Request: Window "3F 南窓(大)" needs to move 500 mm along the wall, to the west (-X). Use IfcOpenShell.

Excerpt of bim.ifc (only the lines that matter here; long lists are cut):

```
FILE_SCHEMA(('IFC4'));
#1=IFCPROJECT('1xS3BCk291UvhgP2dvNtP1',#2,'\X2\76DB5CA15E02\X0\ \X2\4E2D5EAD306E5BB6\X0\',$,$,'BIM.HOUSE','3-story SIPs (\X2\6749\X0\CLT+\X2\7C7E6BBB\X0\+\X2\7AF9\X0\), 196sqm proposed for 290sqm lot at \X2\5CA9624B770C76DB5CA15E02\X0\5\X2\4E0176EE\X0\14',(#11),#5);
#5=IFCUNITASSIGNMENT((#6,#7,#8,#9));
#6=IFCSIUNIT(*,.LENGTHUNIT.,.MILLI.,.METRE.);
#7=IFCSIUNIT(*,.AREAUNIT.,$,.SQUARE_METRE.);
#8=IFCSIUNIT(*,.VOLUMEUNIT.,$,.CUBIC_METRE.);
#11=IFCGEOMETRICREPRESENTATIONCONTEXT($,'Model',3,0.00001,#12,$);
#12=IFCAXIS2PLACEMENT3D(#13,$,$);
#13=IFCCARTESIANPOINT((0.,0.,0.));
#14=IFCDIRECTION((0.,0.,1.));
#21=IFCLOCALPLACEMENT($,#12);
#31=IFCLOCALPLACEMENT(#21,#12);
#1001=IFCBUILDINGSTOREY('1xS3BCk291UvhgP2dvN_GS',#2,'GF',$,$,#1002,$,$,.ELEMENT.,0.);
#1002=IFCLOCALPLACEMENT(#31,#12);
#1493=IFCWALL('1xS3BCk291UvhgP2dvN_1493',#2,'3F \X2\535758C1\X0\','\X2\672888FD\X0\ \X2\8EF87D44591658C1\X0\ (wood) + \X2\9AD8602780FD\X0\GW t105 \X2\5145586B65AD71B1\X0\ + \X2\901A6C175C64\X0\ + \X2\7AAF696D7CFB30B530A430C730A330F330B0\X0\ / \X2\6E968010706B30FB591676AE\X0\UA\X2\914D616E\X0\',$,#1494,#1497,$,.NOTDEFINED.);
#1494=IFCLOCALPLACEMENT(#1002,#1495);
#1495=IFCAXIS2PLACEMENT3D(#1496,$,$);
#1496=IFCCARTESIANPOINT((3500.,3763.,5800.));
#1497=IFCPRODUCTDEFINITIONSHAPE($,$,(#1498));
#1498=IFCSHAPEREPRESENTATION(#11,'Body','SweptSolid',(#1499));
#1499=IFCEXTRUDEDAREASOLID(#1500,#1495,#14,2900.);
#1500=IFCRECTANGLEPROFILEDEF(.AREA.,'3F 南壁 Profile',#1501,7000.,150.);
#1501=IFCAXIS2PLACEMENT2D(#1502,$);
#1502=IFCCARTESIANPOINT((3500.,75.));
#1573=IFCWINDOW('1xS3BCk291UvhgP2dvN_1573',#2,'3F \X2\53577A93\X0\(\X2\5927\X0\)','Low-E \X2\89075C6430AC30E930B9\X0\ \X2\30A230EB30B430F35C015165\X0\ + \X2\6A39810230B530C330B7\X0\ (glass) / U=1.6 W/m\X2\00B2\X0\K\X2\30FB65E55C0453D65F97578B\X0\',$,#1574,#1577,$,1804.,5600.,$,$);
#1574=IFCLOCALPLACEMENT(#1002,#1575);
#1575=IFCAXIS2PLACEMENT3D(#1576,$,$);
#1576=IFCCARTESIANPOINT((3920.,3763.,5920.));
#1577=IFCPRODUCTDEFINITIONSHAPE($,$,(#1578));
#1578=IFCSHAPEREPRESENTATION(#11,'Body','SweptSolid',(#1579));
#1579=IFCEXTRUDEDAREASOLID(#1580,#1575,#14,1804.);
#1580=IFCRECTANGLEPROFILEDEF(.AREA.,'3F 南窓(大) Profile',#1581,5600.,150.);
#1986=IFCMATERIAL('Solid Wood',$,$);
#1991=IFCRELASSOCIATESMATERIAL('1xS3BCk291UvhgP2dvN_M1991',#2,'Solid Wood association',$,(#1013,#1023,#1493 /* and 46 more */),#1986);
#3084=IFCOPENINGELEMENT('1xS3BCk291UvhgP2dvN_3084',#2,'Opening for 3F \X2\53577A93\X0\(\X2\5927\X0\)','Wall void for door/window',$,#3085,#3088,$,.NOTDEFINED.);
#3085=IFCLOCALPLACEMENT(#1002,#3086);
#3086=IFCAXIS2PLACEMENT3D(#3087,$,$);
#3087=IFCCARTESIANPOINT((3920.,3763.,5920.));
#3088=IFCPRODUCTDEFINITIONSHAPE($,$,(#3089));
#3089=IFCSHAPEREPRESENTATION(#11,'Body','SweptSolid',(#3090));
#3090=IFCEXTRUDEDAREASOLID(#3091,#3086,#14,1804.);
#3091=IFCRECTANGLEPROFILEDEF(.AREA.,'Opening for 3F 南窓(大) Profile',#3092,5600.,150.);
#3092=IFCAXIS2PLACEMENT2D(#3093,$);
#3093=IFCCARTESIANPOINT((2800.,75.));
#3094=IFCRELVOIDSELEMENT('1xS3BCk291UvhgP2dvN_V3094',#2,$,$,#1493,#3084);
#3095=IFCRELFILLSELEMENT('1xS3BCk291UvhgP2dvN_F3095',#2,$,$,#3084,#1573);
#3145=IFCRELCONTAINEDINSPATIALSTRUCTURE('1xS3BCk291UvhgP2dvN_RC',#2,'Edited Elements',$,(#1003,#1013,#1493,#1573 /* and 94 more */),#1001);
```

```python
import ifcopenshell
import ifcopenshell.api.geometry
import ifcopenshell.util.placement
import ifcopenshell.util.unit

model = ifcopenshell.open("bim.ifc")
unit_scale = ifcopenshell.util.unit.calculate_unit_scale(model)

window = model.by_guid("1xS3BCk291UvhgP2dvN_1573")
opening = window.FillsVoids[0].RelatingOpeningElement
wall = opening.VoidsElements[0].RelatingBuildingElement

wall_matrix = ifcopenshell.util.placement.get_local_placement(wall.ObjectPlacement)
shift = wall_matrix[:3, 0] * -0.5 / unit_scale
before = ifcopenshell.util.placement.get_local_placement(window.ObjectPlacement)[:3, 3].copy()

# The window is not placed relative to its opening, so move both.
for product in (opening, window):
    matrix = ifcopenshell.util.placement.get_local_placement(product.ObjectPlacement)
    matrix[:3, 3] += shift
    ifcopenshell.api.geometry.edit_object_placement(model, product=product, matrix=matrix, is_si=False)

after = ifcopenshell.util.placement.get_local_placement(window.ObjectPlacement)[:3, 3]
print("window moved by", (after - before).round(3) + 0.0)

model.write("bim_v2.ifc")
```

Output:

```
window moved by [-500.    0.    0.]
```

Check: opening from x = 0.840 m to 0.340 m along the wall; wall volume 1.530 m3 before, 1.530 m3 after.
